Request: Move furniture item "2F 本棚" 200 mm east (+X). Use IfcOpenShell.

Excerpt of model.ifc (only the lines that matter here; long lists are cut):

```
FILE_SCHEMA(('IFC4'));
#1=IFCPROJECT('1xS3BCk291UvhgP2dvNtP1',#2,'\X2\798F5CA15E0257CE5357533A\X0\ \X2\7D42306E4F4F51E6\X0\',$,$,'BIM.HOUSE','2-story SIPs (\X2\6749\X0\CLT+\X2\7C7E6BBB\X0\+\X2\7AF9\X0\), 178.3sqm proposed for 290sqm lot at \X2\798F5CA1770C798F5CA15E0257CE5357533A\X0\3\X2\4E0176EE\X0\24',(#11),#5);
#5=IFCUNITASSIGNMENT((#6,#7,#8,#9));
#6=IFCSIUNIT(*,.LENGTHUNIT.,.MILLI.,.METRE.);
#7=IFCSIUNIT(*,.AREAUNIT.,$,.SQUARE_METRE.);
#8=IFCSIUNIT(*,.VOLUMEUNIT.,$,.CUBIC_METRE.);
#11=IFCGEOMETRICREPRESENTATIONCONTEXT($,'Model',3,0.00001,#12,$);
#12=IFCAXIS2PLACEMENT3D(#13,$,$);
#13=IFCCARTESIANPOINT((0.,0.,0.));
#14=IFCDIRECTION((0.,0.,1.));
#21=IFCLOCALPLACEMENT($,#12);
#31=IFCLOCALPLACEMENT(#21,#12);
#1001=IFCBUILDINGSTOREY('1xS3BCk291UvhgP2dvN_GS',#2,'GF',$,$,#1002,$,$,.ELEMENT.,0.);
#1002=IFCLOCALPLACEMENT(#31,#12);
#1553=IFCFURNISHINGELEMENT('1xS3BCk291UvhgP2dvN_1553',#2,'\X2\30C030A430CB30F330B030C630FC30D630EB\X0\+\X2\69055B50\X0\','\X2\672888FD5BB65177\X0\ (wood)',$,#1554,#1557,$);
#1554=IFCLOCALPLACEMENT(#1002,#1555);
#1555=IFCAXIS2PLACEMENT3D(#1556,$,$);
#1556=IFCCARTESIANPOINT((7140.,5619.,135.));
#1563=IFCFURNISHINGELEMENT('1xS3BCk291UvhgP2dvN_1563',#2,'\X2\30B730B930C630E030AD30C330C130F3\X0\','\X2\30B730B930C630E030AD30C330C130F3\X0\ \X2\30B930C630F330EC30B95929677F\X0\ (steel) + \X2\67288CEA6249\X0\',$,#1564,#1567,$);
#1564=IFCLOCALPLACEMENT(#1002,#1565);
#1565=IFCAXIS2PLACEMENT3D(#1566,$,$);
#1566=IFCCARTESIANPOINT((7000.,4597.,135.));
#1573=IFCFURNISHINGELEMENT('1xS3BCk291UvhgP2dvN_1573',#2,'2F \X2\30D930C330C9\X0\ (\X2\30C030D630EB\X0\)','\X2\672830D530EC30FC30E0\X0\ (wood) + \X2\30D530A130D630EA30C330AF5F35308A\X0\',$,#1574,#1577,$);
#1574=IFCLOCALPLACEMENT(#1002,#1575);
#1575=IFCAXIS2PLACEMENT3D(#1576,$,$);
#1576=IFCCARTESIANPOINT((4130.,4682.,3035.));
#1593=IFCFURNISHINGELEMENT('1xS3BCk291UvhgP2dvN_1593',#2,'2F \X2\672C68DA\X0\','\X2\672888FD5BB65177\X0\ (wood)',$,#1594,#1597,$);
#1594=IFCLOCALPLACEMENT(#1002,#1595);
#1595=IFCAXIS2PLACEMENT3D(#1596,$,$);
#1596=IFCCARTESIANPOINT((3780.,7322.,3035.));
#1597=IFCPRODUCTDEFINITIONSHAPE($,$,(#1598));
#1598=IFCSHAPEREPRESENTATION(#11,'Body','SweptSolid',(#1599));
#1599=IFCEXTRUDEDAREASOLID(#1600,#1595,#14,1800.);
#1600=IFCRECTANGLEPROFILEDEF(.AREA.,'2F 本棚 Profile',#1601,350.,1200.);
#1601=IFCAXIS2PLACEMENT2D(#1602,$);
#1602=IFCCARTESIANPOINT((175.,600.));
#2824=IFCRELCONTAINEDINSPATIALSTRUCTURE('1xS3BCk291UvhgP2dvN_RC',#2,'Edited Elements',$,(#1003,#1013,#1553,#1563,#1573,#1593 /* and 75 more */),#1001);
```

```python
import ifcopenshell
import ifcopenshell.api.geometry
import ifcopenshell.util.placement

model = ifcopenshell.open("model.ifc")

item = model.by_guid("1xS3BCk291UvhgP2dvN_1593")
matrix = ifcopenshell.util.placement.get_local_placement(item.ObjectPlacement)
matrix[0, 3] += 200.0
ifcopenshell.api.geometry.edit_object_placement(model, product=item, matrix=matrix, is_si=False)

print(ifcopenshell.util.placement.get_local_placement(item.ObjectPlacement).round(3) + 0.0)

model.write("model-out.ifc")
```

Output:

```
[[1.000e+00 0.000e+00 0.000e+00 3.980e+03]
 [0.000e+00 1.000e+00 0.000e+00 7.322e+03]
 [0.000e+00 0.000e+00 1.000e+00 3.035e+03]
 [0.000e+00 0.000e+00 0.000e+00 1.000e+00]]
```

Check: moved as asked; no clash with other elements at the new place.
